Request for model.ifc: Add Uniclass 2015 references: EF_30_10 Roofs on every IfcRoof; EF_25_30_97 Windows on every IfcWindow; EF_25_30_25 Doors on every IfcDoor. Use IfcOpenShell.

First a look at what the model holds.

```python
import ifcopenshell

model = ifcopenshell.open("model.ifc")
print(model.schema)
print("classifications:", [c.Name for c in model.by_type("IfcClassification")])
for ifc_class in ("IfcDoor", "IfcRoof", "IfcStair", "IfcWall", "IfcWindow"):
    print(ifc_class, len(model.by_type(ifc_class)))
```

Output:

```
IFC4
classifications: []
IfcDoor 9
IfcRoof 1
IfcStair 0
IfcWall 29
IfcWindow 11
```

```python
import ifcopenshell
import ifcopenshell.api.classification

model = ifcopenshell.open("model.ifc")

system = ifcopenshell.api.classification.add_classification(model, classification="Uniclass 2015")

codes = {
    "IfcRoof": ("EF_30_10", "Roofs"),
    "IfcWindow": ("EF_25_30_97", "Windows"),
    "IfcDoor": ("EF_25_30_25", "Doors"),
}
for ifc_class, (code, name) in codes.items():
    products = model.by_type(ifc_class)
    ifcopenshell.api.classification.add_reference(
        model, products=products, classification=system, identification=code, name=name
    )
    print(code, len(products))

model.write("model_edited.ifc")
```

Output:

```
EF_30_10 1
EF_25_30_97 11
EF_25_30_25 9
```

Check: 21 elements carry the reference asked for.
